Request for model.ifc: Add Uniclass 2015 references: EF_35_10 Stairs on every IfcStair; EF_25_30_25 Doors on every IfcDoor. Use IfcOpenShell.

First a look at what the model holds.

```python
import ifcopenshell

model = ifcopenshell.open("model.ifc")
print(model.schema)
print("classifications:", [c.Name for c in model.by_type("IfcClassification")])
for ifc_class in ("IfcDoor", "IfcRoof", "IfcStair", "IfcWall", "IfcWindow"):
    print(ifc_class, len(model.by_type(ifc_class)))
```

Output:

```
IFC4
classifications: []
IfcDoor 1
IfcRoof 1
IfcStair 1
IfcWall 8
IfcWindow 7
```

```python
import ifcopenshell
import ifcopenshell.api.classification

model = ifcopenshell.open("model.ifc")

system = ifcopenshell.api.classification.add_classification(model, classification="Uniclass 2015")

codes = {
    "IfcStair": ("EF_35_10", "Stairs"),
    "IfcDoor": ("EF_25_30_25", "Doors"),
}
for ifc_class, (code, name) in codes.items():
    products = model.by_type(ifc_class)
    ifcopenshell.api.classification.add_reference(
        model, products=products, classification=system, identification=code, name=name
    )
    print(code, len(products))

model.write("model_v2.ifc")
```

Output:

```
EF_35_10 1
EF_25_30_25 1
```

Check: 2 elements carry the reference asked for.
